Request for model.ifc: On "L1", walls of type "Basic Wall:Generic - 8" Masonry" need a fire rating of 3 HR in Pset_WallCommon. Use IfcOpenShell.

First a look at what the model holds.

```python
import ifcopenshell
import ifcopenshell.util.element

model = ifcopenshell.open("model.ifc")
print(model.schema)
storey = next(s for s in model.by_type("IfcBuildingStorey") if s.Name == "L1")
walls = [e for e in ifcopenshell.util.element.get_decomposition(storey) if e.is_a("IfcWall")]
seen = {}
for e in walls:
    element_type = ifcopenshell.util.element.get_type(e)
    key = (element_type.Name if element_type != e and element_type else None, ifcopenshell.util.element.get_pset(e, "Pset_WallCommon", "FireRating"))
    seen[key] = seen.get(key, 0) + 1
for (name, value), count in sorted(seen.items(), key=str):
    print(count, "x", name, "|", value)
```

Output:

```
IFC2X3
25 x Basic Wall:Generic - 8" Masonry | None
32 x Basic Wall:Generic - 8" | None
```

```python
import ifcopenshell
import ifcopenshell.api.pset
import ifcopenshell.util.element

model = ifcopenshell.open("model.ifc")

storey = next(s for s in model.by_type("IfcBuildingStorey") if s.Name == "L1")
walls = [e for e in ifcopenshell.util.element.get_decomposition(storey) if e.is_a("IfcWall")]

count = 0
for e in walls:
    element_type = ifcopenshell.util.element.get_type(e)
    if element_type in (None, e) or element_type.Name != 'Basic Wall:Generic - 8" Masonry':
        continue
    # add_pset returns the element's existing set when there is one.
    pset = ifcopenshell.api.pset.add_pset(model, product=e, name="Pset_WallCommon")
    ifcopenshell.api.pset.edit_pset(model, pset=pset, properties={"FireRating": "3 HR"})
    count += 1

print(count, "walls updated")

model.write("model_rev.ifc")
```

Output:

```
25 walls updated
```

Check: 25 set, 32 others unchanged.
